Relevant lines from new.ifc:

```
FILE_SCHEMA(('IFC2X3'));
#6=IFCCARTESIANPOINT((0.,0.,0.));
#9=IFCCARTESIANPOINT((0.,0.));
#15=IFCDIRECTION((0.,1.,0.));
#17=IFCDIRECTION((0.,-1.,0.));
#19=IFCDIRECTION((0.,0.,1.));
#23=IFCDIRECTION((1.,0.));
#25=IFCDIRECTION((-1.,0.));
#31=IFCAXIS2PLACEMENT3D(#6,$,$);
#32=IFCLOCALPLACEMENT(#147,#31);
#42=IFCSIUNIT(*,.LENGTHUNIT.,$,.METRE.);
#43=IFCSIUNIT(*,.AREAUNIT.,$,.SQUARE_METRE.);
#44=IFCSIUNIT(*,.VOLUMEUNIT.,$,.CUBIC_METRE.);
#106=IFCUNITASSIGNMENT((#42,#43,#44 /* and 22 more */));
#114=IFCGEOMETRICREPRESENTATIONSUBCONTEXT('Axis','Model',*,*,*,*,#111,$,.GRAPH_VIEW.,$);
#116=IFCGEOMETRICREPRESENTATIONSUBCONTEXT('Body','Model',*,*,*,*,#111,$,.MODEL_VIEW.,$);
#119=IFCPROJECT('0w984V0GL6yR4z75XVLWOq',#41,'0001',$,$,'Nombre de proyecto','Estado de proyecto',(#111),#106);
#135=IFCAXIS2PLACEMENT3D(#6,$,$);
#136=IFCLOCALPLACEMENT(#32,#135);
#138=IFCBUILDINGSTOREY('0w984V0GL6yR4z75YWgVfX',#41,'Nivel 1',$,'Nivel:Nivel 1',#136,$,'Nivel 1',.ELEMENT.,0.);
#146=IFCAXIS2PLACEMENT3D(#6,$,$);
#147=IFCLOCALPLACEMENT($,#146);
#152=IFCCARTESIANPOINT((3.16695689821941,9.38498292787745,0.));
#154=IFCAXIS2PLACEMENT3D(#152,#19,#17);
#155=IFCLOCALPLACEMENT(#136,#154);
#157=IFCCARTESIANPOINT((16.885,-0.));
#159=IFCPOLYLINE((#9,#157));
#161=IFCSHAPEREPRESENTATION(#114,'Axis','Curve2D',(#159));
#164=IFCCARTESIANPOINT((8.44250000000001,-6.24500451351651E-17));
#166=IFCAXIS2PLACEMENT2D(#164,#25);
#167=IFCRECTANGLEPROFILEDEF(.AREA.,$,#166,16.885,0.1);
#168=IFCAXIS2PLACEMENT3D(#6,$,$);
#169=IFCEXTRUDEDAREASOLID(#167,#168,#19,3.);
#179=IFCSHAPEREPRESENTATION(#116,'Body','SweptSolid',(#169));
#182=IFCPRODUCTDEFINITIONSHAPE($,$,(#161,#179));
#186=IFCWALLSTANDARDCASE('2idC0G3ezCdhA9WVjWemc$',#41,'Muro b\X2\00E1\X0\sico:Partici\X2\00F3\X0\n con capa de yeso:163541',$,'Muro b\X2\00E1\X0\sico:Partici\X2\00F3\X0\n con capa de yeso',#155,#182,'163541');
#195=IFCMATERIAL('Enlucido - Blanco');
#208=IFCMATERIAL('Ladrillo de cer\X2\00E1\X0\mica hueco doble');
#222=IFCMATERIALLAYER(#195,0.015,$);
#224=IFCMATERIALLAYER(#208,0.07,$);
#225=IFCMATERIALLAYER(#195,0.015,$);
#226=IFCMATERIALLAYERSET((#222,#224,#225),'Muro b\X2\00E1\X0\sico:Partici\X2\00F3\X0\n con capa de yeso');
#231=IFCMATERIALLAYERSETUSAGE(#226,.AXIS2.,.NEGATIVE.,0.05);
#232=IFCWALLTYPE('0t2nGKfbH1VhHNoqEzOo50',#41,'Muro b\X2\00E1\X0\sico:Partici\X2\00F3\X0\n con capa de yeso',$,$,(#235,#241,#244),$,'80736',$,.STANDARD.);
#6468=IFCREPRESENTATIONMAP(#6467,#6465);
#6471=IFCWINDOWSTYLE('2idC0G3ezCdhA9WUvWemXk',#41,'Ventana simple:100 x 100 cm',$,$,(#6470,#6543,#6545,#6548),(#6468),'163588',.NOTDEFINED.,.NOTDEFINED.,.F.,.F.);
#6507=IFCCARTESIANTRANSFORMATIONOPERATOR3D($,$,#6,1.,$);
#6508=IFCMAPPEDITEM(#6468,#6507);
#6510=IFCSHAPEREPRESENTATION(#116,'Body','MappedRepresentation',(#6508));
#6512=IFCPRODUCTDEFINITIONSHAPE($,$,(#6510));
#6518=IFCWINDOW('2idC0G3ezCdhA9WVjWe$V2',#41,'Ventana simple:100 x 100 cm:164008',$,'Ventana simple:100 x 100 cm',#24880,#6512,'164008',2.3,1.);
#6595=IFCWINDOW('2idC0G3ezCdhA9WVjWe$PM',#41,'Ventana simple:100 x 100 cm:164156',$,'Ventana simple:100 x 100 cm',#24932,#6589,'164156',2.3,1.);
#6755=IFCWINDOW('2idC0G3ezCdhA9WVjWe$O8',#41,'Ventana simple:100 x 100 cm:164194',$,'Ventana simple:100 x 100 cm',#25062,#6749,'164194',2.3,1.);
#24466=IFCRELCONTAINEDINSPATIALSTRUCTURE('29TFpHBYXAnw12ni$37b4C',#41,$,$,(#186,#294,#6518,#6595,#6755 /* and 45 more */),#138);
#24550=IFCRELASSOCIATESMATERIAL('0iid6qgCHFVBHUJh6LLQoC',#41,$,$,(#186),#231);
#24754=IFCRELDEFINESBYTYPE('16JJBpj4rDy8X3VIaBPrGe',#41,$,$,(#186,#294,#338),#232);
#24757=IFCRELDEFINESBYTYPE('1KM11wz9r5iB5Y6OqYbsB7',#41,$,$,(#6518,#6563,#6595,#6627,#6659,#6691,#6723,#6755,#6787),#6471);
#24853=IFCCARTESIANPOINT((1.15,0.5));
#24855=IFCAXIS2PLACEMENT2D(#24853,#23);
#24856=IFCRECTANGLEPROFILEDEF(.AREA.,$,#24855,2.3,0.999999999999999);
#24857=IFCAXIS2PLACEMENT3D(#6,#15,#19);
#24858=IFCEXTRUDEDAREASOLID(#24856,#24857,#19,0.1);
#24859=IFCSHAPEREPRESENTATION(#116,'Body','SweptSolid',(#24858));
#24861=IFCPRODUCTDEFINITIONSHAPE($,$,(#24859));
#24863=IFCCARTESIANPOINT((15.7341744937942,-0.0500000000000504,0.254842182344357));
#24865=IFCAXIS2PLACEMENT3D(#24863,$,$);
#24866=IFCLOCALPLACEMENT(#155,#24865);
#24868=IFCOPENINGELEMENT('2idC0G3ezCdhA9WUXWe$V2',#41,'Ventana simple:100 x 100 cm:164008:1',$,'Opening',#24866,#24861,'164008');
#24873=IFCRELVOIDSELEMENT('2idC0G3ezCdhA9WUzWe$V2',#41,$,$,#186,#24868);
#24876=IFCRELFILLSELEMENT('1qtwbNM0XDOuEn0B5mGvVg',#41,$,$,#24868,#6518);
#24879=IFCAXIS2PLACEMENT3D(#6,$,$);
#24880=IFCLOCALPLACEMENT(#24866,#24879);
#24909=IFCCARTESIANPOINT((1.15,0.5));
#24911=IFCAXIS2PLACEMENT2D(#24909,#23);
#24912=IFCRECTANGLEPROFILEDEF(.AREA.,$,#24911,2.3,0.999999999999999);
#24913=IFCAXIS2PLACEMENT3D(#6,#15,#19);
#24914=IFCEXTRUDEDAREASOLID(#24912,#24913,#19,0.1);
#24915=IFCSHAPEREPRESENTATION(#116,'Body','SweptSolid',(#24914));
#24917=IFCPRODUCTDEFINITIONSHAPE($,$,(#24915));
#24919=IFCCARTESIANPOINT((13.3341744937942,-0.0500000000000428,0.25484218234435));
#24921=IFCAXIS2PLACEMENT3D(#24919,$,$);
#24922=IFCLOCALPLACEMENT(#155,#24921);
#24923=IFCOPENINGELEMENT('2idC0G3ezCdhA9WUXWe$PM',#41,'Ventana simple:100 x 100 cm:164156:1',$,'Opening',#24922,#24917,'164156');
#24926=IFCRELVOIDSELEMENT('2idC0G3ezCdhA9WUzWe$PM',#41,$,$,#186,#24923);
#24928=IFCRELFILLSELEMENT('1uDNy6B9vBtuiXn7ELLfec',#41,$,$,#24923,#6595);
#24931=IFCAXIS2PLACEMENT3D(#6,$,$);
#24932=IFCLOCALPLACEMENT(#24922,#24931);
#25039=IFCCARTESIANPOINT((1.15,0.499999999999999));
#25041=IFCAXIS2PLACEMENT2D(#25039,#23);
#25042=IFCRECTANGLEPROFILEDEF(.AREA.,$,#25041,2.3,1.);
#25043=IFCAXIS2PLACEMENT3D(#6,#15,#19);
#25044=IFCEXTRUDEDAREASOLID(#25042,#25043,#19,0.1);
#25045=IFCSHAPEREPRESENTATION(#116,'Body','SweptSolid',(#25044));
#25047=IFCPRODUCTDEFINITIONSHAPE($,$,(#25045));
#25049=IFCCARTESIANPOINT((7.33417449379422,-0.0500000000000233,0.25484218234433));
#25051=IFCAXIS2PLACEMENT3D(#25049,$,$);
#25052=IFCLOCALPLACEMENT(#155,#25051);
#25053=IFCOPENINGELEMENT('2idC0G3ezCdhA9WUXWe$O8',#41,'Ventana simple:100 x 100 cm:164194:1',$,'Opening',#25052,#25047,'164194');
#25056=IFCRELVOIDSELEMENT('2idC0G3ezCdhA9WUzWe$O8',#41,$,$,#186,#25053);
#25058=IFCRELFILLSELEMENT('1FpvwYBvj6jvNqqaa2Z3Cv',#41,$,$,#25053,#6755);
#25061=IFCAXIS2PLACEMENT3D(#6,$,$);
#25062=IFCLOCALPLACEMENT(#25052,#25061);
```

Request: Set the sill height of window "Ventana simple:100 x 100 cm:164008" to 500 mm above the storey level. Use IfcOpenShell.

```python
import numpy as np
import ifcopenshell
import ifcopenshell.api.geometry
import ifcopenshell.geom
import ifcopenshell.util.element
import ifcopenshell.util.placement
import ifcopenshell.util.shape
import ifcopenshell.util.unit

model = ifcopenshell.open("new.ifc")
unit_scale = ifcopenshell.util.unit.calculate_unit_scale(model)

window = model.by_guid("2idC0G3ezCdhA9WVjWe$V2")
opening = window.FillsVoids[0].RelatingOpeningElement
storey = ifcopenshell.util.element.get_container(window, ifc_class="IfcBuildingStorey")
level = ifcopenshell.util.placement.get_local_placement(storey.ObjectPlacement)[2, 3]

# The opening's origin need not be at the sill, so measure its lowest point.
shape = ifcopenshell.geom.create_shape(ifcopenshell.geom.settings(), opening)
bottom = ifcopenshell.util.shape.get_shape_bottom_elevation(shape, shape.geometry) / unit_scale
dz = level + 0.5 / unit_scale - bottom

shift = np.array([0.0, 0.0, dz])
# The window is placed relative to its opening, so it follows when the opening moves.
matrix = ifcopenshell.util.placement.get_local_placement(opening.ObjectPlacement)
matrix[:3, 3] += shift
ifcopenshell.api.geometry.edit_object_placement(
    model, product=opening, matrix=matrix, is_si=False, should_transform_children=True
)

print(f"moved by {dz * unit_scale:+.3f} m")

model.write("new_edited.ifc")
```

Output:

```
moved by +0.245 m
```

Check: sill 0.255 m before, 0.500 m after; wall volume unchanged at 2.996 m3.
